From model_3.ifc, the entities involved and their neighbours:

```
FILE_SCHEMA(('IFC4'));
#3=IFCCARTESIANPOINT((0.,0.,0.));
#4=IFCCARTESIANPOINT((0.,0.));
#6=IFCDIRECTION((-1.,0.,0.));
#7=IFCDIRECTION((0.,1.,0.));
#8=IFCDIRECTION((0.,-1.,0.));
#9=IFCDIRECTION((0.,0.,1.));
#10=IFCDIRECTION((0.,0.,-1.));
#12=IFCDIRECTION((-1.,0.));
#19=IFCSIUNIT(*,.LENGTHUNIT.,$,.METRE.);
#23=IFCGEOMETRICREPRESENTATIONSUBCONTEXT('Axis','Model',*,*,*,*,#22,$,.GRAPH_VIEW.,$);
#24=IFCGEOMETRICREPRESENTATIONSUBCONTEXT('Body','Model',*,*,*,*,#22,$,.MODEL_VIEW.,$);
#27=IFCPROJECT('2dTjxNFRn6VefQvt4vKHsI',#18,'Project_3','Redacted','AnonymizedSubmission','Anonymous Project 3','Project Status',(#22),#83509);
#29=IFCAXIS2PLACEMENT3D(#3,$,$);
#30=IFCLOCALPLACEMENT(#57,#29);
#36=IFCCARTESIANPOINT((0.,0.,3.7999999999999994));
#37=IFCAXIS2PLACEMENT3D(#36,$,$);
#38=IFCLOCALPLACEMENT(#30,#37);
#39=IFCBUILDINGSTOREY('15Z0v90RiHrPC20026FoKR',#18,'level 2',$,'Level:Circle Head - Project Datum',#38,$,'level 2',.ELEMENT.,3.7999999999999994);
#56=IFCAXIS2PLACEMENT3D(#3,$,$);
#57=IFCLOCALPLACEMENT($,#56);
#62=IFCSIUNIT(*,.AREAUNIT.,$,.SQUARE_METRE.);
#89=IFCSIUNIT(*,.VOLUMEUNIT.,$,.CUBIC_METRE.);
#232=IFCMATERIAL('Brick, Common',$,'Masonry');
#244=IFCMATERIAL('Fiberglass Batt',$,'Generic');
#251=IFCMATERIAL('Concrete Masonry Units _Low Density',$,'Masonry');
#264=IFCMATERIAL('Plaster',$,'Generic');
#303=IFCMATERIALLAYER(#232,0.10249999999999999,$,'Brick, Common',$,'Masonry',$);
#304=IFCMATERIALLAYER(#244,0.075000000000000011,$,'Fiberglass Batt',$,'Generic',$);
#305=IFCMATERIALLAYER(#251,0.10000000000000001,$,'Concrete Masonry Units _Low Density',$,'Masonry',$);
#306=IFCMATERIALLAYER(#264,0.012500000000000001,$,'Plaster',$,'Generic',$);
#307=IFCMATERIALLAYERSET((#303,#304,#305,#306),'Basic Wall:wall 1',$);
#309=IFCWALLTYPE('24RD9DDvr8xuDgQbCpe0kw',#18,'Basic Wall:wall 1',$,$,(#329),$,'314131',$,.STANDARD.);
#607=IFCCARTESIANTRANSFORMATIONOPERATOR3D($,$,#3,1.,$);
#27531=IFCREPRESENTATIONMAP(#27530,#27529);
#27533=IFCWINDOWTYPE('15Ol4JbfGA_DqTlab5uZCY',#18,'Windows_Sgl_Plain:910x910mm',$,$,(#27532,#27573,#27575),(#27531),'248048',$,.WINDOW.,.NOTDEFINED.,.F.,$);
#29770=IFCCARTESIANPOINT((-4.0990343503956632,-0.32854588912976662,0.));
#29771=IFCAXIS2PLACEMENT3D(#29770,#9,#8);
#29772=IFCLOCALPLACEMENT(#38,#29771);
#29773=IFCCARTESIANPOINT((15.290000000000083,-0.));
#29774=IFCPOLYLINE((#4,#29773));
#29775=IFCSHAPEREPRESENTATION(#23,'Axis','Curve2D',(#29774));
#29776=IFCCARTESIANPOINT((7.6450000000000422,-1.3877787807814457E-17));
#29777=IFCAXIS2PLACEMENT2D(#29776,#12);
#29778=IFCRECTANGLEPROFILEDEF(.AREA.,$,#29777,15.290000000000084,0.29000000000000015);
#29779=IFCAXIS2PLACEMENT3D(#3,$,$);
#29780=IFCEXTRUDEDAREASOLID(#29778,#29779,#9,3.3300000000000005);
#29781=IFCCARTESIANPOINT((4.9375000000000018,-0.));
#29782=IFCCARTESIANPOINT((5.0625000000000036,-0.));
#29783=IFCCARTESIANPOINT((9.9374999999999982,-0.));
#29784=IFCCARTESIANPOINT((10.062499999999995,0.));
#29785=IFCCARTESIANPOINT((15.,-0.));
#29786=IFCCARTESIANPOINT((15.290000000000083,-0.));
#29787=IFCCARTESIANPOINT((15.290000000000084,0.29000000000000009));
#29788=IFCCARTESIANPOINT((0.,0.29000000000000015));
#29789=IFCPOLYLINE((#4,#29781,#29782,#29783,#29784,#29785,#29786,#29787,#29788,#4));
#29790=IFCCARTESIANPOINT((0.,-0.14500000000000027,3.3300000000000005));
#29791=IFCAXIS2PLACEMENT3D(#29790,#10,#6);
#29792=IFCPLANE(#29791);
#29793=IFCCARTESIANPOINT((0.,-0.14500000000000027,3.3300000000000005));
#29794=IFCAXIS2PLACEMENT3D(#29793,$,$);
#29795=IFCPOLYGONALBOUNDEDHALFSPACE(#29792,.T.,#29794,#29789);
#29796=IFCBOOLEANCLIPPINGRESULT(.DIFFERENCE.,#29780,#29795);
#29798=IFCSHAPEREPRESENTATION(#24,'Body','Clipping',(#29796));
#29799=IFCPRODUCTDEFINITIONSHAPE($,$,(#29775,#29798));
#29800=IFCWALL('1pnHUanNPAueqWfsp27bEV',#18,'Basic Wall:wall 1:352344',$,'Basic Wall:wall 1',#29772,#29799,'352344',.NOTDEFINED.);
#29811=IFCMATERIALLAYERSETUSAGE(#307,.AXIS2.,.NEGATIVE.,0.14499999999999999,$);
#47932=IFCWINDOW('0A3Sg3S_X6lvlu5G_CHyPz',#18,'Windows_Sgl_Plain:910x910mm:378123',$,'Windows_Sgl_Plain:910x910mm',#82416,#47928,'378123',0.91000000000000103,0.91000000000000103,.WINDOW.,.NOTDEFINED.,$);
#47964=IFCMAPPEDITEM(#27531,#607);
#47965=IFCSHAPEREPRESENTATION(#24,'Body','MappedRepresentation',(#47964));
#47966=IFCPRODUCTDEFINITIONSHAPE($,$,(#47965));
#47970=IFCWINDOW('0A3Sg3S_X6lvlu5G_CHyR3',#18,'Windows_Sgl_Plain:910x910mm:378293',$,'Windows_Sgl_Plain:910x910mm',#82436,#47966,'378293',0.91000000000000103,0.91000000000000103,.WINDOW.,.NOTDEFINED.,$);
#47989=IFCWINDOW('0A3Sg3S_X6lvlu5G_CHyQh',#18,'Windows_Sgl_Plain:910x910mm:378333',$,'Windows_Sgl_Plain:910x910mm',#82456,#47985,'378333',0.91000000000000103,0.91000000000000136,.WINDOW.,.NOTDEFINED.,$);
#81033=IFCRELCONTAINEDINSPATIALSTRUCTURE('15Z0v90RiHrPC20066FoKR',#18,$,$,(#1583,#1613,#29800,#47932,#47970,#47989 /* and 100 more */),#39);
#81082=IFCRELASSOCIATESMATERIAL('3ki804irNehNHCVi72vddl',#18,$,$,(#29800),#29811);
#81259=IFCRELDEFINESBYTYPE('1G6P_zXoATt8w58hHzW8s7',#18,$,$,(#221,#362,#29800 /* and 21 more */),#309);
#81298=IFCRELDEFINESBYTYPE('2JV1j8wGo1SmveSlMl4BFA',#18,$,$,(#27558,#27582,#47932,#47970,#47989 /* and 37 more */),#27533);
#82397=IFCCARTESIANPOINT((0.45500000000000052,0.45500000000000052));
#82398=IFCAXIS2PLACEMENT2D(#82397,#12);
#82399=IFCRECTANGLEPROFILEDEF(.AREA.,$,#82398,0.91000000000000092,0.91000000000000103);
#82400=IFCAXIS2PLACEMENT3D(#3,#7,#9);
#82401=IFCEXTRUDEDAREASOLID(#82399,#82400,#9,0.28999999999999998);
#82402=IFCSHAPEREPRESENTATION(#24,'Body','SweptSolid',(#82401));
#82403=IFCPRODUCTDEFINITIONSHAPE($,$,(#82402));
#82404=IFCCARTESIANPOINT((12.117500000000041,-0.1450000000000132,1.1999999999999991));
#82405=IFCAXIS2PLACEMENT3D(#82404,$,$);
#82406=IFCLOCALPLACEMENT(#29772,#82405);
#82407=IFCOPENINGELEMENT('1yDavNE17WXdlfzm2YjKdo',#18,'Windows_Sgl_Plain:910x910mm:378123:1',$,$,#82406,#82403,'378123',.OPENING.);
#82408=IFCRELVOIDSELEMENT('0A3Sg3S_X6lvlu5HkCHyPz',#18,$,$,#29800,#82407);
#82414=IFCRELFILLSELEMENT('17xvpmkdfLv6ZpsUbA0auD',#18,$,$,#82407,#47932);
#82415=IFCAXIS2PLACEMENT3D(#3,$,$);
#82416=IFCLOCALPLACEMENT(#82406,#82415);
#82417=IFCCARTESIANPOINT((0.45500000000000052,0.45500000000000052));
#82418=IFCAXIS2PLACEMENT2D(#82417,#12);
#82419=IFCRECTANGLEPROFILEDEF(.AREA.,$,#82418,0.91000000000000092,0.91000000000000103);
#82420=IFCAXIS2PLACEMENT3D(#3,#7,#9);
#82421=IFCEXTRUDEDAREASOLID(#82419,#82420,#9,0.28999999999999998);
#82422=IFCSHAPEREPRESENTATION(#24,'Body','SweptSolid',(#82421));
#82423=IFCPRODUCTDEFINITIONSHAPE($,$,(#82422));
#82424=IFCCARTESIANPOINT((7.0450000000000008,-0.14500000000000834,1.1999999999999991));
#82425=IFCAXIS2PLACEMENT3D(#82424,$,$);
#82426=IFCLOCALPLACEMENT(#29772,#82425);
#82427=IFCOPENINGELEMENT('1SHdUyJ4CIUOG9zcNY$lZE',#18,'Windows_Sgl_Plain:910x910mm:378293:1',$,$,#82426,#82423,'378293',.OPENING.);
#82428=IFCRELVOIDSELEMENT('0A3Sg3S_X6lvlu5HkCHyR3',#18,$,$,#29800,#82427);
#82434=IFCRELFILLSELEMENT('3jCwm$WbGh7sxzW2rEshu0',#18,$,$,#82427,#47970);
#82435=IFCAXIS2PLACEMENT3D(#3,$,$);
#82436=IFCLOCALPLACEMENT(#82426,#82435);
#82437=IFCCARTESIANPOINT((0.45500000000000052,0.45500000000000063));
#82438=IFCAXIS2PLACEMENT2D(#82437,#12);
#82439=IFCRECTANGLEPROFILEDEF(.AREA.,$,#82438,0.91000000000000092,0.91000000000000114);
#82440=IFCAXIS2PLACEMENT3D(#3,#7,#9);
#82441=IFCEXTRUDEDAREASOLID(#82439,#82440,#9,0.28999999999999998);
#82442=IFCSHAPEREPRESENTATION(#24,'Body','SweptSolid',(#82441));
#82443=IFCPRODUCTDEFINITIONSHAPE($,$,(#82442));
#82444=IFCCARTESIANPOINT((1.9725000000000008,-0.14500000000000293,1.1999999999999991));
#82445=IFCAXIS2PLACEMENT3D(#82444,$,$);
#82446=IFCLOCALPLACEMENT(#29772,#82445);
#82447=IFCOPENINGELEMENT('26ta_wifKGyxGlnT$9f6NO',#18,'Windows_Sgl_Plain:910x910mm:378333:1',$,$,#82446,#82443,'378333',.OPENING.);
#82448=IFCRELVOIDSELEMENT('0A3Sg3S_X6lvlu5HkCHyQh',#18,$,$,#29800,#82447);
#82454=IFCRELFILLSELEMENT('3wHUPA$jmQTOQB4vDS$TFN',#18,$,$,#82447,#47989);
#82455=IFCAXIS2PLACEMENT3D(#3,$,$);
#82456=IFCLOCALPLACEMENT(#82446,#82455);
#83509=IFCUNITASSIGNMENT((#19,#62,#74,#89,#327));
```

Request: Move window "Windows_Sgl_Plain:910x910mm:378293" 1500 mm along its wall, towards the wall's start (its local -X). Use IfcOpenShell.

```python
import ifcopenshell
import ifcopenshell.api.geometry
import ifcopenshell.util.placement
import ifcopenshell.util.unit

model = ifcopenshell.open("model_3.ifc")
unit_scale = ifcopenshell.util.unit.calculate_unit_scale(model)

window = model.by_id(47970)
opening = window.FillsVoids[0].RelatingOpeningElement
wall = opening.VoidsElements[0].RelatingBuildingElement

wall_matrix = ifcopenshell.util.placement.get_local_placement(wall.ObjectPlacement)
shift = wall_matrix[:3, 0] * -1.5 / unit_scale
before = ifcopenshell.util.placement.get_local_placement(window.ObjectPlacement)[:3, 3].copy()

# The window is placed relative to its opening, so it follows when the opening moves.
matrix = ifcopenshell.util.placement.get_local_placement(opening.ObjectPlacement)
matrix[:3, 3] += shift
ifcopenshell.api.geometry.edit_object_placement(
    model, product=opening, matrix=matrix, is_si=False, should_transform_children=True
)

after = ifcopenshell.util.placement.get_local_placement(window.ObjectPlacement)[:3, 3]
print("window moved by", (after - before).round(3) + 0.0)

model.write("model_3_edited.ifc")
```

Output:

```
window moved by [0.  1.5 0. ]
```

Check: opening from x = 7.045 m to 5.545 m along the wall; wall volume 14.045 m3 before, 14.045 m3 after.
